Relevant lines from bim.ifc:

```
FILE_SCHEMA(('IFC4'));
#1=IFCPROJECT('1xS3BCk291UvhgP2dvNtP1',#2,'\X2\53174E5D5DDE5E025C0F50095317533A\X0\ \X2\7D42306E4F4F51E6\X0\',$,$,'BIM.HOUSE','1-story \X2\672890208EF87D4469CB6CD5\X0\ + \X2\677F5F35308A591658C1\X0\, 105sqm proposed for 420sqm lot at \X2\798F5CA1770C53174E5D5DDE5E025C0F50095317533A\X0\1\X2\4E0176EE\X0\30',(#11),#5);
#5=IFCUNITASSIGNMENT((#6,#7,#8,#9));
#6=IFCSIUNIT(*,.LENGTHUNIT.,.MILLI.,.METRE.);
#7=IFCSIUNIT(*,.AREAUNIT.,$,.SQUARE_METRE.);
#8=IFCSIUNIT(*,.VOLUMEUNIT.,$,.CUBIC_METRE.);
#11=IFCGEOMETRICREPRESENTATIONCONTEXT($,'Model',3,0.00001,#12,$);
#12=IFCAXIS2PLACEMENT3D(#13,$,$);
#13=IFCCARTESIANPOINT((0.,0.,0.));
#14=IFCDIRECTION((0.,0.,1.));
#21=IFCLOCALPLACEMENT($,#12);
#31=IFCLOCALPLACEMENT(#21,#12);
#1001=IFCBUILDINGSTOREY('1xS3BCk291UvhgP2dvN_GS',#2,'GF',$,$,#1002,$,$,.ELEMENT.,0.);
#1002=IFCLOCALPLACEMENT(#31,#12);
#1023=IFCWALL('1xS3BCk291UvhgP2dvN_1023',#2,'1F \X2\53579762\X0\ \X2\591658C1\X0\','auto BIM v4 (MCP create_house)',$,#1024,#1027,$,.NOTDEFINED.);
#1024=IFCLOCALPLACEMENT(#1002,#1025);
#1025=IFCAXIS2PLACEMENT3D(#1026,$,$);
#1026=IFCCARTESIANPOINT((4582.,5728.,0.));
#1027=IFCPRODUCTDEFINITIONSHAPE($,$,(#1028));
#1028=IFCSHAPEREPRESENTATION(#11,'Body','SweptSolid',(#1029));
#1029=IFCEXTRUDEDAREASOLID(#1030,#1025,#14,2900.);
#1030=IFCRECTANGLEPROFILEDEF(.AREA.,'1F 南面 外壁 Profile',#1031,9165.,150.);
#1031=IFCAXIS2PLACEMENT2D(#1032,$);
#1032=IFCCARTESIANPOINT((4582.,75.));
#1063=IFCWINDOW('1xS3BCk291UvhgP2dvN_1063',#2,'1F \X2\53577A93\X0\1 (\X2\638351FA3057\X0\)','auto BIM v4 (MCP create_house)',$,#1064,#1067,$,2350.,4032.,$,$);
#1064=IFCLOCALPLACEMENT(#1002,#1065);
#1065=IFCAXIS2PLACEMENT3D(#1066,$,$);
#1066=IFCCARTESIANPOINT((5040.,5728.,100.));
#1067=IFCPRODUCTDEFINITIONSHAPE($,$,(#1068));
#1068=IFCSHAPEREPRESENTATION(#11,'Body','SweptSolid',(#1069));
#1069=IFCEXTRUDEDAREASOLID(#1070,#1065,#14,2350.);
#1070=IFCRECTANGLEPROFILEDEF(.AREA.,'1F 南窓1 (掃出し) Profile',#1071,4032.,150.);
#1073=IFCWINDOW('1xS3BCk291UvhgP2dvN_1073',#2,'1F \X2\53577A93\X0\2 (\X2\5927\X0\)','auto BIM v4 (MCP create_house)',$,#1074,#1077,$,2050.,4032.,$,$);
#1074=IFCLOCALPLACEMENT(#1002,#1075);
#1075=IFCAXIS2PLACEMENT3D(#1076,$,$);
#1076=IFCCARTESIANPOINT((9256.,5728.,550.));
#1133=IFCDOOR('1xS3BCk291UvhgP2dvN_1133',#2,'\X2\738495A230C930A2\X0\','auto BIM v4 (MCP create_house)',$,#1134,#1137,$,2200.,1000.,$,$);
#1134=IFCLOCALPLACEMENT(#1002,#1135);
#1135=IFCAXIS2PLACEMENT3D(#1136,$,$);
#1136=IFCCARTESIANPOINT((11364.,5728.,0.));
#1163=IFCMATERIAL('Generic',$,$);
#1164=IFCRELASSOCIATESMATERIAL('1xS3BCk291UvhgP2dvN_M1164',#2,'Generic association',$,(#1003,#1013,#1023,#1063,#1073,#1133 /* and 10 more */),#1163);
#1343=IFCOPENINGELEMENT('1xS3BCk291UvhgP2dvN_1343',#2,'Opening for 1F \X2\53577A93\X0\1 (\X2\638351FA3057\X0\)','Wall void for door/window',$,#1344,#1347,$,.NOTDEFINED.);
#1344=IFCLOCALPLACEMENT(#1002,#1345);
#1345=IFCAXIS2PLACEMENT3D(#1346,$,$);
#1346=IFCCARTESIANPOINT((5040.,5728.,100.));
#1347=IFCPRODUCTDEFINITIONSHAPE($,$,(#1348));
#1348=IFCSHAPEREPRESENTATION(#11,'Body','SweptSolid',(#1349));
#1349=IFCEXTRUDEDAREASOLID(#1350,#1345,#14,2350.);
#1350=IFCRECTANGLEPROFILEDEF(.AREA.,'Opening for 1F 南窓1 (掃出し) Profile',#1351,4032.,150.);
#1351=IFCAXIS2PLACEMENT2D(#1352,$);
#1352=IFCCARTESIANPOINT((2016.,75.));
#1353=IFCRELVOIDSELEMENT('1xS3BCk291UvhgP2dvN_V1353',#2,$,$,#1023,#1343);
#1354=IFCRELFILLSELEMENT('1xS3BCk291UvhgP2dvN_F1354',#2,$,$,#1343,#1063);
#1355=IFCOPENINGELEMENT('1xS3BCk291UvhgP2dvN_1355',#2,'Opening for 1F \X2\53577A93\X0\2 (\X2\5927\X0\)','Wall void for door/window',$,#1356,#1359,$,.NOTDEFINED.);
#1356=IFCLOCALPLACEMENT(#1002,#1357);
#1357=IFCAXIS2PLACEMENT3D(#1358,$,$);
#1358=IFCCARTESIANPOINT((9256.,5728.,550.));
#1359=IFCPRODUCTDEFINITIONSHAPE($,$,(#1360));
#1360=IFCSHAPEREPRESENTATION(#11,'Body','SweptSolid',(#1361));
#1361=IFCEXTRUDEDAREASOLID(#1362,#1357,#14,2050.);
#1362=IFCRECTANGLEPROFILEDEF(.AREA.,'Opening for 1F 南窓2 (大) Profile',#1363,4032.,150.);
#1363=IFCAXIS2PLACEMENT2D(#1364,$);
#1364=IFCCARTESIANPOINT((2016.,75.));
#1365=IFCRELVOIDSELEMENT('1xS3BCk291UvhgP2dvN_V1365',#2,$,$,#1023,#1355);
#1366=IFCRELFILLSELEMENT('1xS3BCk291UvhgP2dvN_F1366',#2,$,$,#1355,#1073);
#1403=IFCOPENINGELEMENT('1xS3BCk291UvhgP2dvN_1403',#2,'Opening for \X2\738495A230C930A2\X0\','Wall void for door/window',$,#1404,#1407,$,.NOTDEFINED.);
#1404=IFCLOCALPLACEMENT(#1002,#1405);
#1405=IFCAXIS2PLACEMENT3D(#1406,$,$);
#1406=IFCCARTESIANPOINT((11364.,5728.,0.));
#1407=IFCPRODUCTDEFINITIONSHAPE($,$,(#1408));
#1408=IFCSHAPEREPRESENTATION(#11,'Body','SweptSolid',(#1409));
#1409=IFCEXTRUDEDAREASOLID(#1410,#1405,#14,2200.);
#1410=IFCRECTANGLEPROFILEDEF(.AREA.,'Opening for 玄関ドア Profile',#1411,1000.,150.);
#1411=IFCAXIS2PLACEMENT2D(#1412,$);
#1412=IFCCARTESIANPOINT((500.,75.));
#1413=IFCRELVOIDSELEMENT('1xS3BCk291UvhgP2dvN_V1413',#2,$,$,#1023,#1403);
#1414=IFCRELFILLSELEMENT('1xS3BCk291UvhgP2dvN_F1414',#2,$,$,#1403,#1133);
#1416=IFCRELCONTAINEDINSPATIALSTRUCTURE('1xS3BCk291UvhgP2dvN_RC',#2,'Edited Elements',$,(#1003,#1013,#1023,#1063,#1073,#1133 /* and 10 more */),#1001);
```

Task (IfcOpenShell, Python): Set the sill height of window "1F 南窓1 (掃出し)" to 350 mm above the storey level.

```python
import numpy as np
import ifcopenshell
import ifcopenshell.api.geometry
import ifcopenshell.geom
import ifcopenshell.util.element
import ifcopenshell.util.placement
import ifcopenshell.util.shape
import ifcopenshell.util.unit

model = ifcopenshell.open("bim.ifc")
unit_scale = ifcopenshell.util.unit.calculate_unit_scale(model)

window = model.by_guid("1xS3BCk291UvhgP2dvN_1063")
opening = window.FillsVoids[0].RelatingOpeningElement
storey = ifcopenshell.util.element.get_container(window, ifc_class="IfcBuildingStorey")
level = ifcopenshell.util.placement.get_local_placement(storey.ObjectPlacement)[2, 3]

# The opening's origin need not be at the sill, so measure its lowest point.
shape = ifcopenshell.geom.create_shape(ifcopenshell.geom.settings(), opening)
bottom = ifcopenshell.util.shape.get_shape_bottom_elevation(shape, shape.geometry) / unit_scale
dz = level + 0.35 / unit_scale - bottom

shift = np.array([0.0, 0.0, dz])
# The window is not placed relative to its opening, so move both.
for product in (opening, window):
    matrix = ifcopenshell.util.placement.get_local_placement(product.ObjectPlacement)
    matrix[:3, 3] += shift
    ifcopenshell.api.geometry.edit_object_placement(model, product=product, matrix=matrix, is_si=False)

print(f"moved by {dz * unit_scale:+.3f} m")

model.write("bim-out.ifc")
```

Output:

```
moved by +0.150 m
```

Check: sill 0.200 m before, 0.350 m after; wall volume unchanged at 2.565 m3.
